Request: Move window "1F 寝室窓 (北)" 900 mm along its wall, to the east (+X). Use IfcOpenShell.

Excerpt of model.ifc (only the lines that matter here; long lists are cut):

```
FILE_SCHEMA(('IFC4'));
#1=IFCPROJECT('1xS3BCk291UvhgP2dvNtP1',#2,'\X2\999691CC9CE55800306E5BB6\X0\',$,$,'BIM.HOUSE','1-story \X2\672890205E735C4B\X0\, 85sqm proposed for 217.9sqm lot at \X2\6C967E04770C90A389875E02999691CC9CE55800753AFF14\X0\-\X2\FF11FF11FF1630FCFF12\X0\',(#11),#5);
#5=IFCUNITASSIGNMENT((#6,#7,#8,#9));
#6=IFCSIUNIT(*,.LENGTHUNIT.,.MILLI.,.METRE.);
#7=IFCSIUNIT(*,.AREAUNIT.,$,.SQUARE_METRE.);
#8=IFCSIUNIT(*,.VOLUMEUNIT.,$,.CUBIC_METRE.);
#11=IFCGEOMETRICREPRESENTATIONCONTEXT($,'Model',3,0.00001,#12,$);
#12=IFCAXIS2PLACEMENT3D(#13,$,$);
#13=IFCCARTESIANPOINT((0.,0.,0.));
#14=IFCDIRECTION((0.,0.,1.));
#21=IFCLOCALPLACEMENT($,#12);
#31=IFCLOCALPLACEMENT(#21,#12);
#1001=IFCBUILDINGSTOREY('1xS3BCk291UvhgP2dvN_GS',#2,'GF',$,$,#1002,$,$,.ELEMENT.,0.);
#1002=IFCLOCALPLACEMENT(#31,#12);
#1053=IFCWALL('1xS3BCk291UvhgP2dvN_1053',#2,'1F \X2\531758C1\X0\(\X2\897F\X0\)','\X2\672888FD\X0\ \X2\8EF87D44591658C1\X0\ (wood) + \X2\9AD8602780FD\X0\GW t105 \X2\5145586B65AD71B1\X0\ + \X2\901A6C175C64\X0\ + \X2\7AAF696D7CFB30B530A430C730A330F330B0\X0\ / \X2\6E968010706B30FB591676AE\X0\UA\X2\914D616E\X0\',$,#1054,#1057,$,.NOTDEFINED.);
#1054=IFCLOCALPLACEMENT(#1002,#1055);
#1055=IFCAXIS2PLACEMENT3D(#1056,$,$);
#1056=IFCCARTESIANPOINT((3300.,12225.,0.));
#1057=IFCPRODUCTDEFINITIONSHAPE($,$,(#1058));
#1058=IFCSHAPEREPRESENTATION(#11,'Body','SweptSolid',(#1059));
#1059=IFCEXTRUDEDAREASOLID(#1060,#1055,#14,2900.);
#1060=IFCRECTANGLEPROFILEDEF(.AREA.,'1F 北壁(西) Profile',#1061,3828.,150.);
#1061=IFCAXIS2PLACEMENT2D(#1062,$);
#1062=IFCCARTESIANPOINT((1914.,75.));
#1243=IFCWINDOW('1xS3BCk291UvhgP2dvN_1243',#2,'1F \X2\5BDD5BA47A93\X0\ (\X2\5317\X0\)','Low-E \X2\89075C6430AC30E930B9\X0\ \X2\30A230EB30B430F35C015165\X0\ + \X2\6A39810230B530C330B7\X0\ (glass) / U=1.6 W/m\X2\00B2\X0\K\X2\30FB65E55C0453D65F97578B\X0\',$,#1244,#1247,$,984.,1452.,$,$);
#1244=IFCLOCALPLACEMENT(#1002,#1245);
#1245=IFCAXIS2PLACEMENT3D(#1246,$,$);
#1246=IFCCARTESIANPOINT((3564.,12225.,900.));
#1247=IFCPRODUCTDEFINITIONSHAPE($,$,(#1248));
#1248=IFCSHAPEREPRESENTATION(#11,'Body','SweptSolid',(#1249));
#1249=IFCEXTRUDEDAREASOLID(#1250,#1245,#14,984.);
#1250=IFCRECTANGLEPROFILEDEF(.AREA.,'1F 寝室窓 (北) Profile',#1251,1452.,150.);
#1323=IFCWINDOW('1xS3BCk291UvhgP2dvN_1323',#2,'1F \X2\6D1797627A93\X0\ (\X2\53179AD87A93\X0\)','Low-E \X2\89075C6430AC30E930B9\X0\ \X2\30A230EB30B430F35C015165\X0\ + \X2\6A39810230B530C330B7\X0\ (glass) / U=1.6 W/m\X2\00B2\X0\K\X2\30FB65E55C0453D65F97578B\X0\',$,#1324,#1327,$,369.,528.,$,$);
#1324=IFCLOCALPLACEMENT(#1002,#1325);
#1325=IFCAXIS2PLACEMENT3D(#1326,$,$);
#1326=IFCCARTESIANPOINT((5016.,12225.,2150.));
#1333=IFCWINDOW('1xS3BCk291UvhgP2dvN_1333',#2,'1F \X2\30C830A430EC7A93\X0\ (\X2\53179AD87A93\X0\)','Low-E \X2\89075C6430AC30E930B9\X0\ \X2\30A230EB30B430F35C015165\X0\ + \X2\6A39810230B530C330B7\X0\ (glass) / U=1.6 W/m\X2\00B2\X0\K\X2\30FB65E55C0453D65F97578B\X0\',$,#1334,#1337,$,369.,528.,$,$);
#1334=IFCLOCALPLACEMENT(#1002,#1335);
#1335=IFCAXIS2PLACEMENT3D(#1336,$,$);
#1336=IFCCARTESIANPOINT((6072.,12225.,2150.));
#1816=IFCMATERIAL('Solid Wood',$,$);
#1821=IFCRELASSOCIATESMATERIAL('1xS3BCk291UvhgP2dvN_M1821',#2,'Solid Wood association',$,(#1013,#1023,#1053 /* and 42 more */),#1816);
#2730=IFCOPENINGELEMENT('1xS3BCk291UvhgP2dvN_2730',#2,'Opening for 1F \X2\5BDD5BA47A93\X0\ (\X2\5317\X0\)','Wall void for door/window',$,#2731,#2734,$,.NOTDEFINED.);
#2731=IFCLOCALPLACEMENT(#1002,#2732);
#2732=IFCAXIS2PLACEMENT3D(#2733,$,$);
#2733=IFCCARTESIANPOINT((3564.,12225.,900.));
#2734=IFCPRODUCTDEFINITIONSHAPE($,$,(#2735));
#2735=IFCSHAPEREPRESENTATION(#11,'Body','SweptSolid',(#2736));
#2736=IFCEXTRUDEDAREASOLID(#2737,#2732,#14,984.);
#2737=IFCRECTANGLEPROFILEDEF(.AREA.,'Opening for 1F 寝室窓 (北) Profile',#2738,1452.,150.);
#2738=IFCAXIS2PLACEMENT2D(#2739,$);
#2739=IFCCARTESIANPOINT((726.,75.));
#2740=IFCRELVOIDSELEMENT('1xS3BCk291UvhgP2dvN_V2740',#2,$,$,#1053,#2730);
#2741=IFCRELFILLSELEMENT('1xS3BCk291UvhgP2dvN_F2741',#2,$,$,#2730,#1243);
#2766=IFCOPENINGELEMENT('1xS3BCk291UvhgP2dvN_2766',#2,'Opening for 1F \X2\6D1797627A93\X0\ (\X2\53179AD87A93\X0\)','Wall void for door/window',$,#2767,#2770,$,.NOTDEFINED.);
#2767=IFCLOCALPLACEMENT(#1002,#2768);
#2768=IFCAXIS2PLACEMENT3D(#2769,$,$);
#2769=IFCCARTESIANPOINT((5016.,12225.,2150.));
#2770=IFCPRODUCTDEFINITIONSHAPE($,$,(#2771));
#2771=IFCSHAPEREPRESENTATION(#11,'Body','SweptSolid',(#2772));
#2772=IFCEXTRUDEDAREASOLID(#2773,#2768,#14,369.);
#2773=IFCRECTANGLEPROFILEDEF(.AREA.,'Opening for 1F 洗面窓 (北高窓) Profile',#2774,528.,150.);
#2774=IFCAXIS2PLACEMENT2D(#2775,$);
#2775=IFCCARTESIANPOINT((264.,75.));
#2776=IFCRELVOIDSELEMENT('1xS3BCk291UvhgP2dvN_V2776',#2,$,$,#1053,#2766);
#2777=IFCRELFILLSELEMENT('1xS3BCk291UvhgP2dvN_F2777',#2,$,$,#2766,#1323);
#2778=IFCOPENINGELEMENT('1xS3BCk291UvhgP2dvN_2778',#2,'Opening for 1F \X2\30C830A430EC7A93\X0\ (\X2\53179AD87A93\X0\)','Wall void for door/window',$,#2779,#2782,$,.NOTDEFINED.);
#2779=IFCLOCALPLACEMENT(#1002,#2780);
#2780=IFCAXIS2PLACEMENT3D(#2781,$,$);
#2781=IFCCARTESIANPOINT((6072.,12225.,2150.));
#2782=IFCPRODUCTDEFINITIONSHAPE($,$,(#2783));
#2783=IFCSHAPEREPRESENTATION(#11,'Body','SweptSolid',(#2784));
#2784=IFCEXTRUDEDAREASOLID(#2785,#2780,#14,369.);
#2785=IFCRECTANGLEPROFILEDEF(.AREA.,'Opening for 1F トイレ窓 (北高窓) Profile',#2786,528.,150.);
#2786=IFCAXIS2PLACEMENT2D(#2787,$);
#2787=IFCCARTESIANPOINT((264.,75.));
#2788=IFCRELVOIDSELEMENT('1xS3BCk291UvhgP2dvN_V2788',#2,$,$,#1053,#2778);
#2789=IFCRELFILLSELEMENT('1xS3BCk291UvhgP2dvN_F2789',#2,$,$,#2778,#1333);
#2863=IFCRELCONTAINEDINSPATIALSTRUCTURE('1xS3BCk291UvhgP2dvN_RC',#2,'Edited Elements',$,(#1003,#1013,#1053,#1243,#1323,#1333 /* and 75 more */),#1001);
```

```python
import ifcopenshell
import ifcopenshell.api.geometry
import ifcopenshell.util.placement
import ifcopenshell.util.unit

model = ifcopenshell.open("model.ifc")
unit_scale = ifcopenshell.util.unit.calculate_unit_scale(model)

window = model.by_guid("1xS3BCk291UvhgP2dvN_1243")
opening = window.FillsVoids[0].RelatingOpeningElement
wall = opening.VoidsElements[0].RelatingBuildingElement

wall_matrix = ifcopenshell.util.placement.get_local_placement(wall.ObjectPlacement)
shift = wall_matrix[:3, 0] * 0.9 / unit_scale
before = ifcopenshell.util.placement.get_local_placement(window.ObjectPlacement)[:3, 3].copy()

# The window is not placed relative to its opening, so move both.
for product in (opening, window):
    matrix = ifcopenshell.util.placement.get_local_placement(product.ObjectPlacement)
    matrix[:3, 3] += shift
    ifcopenshell.api.geometry.edit_object_placement(model, product=product, matrix=matrix, is_si=False)

after = ifcopenshell.util.placement.get_local_placement(window.ObjectPlacement)[:3, 3]
print("window moved by", (after - before).round(3) + 0.0)

model.write("model_edited.ifc")
```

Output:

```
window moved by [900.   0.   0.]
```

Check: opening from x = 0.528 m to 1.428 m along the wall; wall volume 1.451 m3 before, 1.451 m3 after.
